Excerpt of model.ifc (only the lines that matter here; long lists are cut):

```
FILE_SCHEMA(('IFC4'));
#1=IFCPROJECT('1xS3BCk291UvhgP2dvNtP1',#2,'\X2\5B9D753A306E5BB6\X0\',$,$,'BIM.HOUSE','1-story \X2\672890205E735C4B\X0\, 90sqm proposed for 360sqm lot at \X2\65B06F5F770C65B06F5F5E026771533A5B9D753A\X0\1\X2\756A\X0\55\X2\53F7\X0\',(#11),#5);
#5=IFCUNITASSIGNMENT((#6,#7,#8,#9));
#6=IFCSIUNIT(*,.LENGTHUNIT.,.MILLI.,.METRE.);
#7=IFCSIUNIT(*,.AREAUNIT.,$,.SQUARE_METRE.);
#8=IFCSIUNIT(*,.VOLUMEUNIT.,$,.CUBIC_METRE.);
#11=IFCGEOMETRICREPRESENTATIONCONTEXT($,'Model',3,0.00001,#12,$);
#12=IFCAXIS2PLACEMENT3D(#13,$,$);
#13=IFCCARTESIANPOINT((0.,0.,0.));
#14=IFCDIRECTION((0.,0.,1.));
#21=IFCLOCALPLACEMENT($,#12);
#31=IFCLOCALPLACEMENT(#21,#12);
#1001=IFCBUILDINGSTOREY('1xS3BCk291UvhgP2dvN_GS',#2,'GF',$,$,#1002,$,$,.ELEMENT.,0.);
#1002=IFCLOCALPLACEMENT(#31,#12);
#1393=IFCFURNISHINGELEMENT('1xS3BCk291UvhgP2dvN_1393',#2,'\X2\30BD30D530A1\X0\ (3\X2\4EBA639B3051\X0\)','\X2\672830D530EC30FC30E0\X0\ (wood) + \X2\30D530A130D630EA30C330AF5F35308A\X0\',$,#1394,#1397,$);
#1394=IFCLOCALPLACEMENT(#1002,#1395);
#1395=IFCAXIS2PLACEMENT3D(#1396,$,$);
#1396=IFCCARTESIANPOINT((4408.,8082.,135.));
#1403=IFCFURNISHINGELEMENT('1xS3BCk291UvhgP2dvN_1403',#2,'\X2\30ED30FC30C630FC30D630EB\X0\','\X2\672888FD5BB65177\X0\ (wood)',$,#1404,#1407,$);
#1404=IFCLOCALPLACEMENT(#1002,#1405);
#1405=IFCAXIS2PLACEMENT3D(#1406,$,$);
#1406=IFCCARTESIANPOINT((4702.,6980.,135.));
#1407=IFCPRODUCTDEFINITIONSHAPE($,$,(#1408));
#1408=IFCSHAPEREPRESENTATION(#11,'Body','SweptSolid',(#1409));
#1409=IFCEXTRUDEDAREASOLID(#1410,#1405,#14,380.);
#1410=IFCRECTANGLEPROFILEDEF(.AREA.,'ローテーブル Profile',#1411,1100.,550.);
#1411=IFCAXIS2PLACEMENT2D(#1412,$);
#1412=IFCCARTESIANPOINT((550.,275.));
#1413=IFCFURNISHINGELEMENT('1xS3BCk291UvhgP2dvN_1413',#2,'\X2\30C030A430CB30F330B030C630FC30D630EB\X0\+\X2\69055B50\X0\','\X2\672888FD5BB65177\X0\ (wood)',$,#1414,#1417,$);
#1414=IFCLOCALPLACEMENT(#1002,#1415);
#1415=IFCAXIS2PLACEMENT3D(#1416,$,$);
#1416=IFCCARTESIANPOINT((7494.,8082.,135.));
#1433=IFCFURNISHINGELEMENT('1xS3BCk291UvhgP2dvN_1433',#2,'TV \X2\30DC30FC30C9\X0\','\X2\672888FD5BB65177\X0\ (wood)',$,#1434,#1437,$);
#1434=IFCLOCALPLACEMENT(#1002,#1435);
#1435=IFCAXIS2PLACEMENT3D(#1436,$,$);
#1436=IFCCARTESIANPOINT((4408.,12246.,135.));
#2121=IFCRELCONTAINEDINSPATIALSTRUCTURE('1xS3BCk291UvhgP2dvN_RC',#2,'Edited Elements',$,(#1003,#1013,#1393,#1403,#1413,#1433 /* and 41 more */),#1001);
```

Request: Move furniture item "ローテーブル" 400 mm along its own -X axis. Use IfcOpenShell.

```python
import ifcopenshell
import ifcopenshell.api.geometry
import ifcopenshell.util.placement

model = ifcopenshell.open("model.ifc")

item = model.by_guid("1xS3BCk291UvhgP2dvN_1403")
matrix = ifcopenshell.util.placement.get_local_placement(item.ObjectPlacement)
matrix[:3, 3] -= matrix[:3, 0] * 400.0
ifcopenshell.api.geometry.edit_object_placement(model, product=item, matrix=matrix, is_si=False)

print(ifcopenshell.util.placement.get_local_placement(item.ObjectPlacement).round(3) + 0.0)

model.write("model_v2.ifc")
```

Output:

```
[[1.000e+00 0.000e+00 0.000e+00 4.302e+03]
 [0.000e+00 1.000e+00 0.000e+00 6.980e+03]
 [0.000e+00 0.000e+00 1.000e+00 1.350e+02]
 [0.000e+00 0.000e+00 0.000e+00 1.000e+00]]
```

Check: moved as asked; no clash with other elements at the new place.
